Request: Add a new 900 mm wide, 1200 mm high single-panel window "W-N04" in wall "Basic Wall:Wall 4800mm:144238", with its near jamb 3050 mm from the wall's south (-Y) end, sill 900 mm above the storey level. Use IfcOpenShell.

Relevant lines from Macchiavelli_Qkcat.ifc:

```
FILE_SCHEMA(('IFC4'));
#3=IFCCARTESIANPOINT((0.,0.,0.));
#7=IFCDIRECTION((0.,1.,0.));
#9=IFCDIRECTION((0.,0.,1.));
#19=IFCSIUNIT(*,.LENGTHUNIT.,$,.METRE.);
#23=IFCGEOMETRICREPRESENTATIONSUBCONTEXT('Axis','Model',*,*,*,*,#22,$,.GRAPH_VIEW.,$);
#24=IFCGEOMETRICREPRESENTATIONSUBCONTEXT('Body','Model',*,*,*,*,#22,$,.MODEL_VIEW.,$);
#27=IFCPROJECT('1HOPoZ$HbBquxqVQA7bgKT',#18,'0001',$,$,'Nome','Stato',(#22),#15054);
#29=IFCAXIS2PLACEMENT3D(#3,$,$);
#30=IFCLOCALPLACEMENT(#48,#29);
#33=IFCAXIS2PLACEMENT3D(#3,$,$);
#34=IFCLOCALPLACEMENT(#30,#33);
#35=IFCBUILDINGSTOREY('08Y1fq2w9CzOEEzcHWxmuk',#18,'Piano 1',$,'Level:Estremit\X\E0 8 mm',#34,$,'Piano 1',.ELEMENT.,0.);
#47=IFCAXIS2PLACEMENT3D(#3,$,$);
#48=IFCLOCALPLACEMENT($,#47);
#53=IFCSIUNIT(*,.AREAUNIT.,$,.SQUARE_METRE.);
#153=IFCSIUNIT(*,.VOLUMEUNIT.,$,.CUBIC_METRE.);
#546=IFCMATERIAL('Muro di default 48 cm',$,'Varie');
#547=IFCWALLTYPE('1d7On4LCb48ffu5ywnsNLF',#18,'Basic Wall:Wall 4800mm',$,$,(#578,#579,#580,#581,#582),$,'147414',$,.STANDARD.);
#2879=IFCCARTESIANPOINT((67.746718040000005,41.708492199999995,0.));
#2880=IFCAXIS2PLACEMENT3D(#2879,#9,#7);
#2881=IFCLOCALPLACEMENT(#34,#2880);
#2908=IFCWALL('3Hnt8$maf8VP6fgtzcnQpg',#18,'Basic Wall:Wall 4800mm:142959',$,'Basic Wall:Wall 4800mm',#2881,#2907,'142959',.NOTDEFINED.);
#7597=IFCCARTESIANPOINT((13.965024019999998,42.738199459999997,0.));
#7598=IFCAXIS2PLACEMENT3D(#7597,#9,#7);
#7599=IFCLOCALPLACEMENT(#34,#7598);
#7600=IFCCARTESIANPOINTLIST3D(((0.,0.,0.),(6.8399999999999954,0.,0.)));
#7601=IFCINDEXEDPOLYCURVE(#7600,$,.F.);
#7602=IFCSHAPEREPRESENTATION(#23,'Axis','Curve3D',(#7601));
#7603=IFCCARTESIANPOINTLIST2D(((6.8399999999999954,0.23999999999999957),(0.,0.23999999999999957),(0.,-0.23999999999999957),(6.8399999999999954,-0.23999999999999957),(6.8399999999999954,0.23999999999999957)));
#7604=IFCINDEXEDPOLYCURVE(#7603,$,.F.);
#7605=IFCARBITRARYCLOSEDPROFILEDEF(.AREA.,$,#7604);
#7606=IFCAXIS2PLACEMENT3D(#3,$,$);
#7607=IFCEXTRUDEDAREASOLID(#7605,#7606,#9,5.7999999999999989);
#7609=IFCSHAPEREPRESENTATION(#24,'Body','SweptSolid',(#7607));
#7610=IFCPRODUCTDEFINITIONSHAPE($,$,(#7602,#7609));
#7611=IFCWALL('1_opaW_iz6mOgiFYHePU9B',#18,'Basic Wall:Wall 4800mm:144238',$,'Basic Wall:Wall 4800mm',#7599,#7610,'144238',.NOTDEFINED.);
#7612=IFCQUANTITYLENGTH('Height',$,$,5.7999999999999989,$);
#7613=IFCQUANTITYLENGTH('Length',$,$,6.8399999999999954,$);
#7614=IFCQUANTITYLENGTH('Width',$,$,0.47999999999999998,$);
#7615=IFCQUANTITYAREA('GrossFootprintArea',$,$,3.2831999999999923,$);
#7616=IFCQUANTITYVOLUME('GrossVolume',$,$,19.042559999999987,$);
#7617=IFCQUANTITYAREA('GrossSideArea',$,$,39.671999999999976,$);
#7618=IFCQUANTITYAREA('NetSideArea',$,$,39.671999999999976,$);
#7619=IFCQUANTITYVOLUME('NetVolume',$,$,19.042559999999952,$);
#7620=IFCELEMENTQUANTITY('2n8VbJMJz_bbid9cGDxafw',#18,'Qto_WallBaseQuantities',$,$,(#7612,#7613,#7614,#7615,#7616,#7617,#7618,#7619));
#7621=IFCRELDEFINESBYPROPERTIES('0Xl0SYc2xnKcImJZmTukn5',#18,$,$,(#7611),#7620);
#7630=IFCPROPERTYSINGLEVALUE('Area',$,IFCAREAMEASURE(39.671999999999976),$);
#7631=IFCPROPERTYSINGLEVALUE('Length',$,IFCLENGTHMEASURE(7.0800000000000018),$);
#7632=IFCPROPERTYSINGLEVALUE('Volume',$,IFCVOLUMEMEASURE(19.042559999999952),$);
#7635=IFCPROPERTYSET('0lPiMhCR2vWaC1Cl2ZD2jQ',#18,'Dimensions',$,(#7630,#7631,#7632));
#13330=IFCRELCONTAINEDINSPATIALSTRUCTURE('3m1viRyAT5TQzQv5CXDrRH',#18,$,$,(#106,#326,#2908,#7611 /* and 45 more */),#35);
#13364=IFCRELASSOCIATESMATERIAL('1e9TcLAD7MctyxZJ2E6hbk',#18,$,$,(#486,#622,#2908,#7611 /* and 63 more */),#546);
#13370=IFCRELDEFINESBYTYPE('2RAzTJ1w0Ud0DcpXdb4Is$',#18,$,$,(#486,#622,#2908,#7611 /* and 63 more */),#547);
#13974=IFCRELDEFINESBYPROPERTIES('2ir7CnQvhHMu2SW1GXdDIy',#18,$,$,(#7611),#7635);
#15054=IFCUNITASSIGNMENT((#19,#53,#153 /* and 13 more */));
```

```python
import numpy as np
import ifcopenshell
import ifcopenshell.api.feature
import ifcopenshell.api.geometry
import ifcopenshell.api.pset
import ifcopenshell.api.root
import ifcopenshell.api.spatial
import ifcopenshell.geom
import ifcopenshell.util.element
import ifcopenshell.util.placement
import ifcopenshell.util.representation
import ifcopenshell.util.shape
import ifcopenshell.util.unit

model = ifcopenshell.open("Macchiavelli_Qkcat.ifc")
unit_scale = ifcopenshell.util.unit.calculate_unit_scale(model)
area_scale = ifcopenshell.util.unit.calculate_unit_scale(model, "AREAUNIT")
volume_scale = ifcopenshell.util.unit.calculate_unit_scale(model, "VOLUMEUNIT")
settings = ifcopenshell.geom.settings()


def volume(element):
    """Net volume in cubic metres, openings subtracted."""
    shape = ifcopenshell.geom.create_shape(settings, element)
    return ifcopenshell.util.shape.get_volume(shape.geometry)


wall = model.by_guid("1_opaW_iz6mOgiFYHePU9B")
storey = ifcopenshell.util.element.get_container(wall, ifc_class="IfcBuildingStorey")
context = ifcopenshell.util.representation.get_context(model, "Model", "Body", "MODEL_VIEW")
before = volume(wall)

width, height, from_end, sill = 0.9, 1.2, 3.05, 0.9  # metres

# The wall runs along its own X axis, and the end named is its -X end.
wall_shape = ifcopenshell.geom.create_shape(settings, wall)
x, y, z = ifcopenshell.util.shape.get_vertices(wall_shape.geometry).T
start = x.min() + from_end
face, thickness = float(y.min()), float(y.max() - y.min())
wall_matrix = ifcopenshell.util.placement.get_local_placement(wall.ObjectPlacement)
level = ifcopenshell.util.placement.get_local_placement(storey.ObjectPlacement)[2, 3]


def in_wall(x, y):
    """Placement at x, y metres in the wall's axes, at sill height."""
    matrix = wall_matrix.copy()
    matrix[:, 3] = wall_matrix @ np.array([x / unit_scale, y / unit_scale, 0.0, 1.0])
    matrix[2, 3] = level + sill / unit_scale
    return matrix


# Opening: a box that overshoots both wall faces by 50 mm.
opening = ifcopenshell.api.root.create_entity(model, ifc_class="IfcOpeningElement", predefined_type="OPENING")
box = ifcopenshell.api.geometry.add_wall_representation(
    model, context=context, length=width, height=height, thickness=thickness + 0.1
)
ifcopenshell.api.geometry.assign_representation(model, product=opening, representation=box)
ifcopenshell.api.geometry.edit_object_placement(model, product=opening, matrix=in_wall(start, face - 0.05), is_si=False)
ifcopenshell.api.feature.add_feature(model, feature=opening, element=wall)

window = ifcopenshell.api.root.create_entity(model, ifc_class="IfcWindow", name="W-N04", predefined_type="WINDOW")
window.OverallWidth, window.OverallHeight = width / unit_scale, height / unit_scale
window.PartitioningType = "SINGLE_PANEL"
body = ifcopenshell.api.geometry.add_window_representation(
    model,
    context=context,
    overall_width=window.OverallWidth,
    overall_height=window.OverallHeight,
    partition_type="SINGLE_PANEL",
)
ifcopenshell.api.geometry.assign_representation(model, product=window, representation=body)
ifcopenshell.api.spatial.assign_container(model, products=[window], relating_structure=storey)
ifcopenshell.api.feature.add_filling(model, opening=opening, element=window)

# Centre the window in the wall's thickness.
ifcopenshell.api.geometry.edit_object_placement(model, product=window, matrix=in_wall(start, face), is_si=False)
window_shape = ifcopenshell.geom.create_shape(settings, window)
depth = ifcopenshell.util.shape.get_vertices(window_shape.geometry)[:, 1]
offset = face + thickness / 2 - (depth.min() + depth.max()) / 2
ifcopenshell.api.geometry.edit_object_placement(model, product=window, matrix=in_wall(start, offset), is_si=False)

after = volume(wall)

# Update the wall's stored quantities.
qto = model.by_id(ifcopenshell.util.element.get_pset(wall, "Qto_WallBaseQuantities", should_inherit=False)["id"])
ifcopenshell.api.pset.edit_qto(model, qto=qto, properties={
    "NetSideArea": after / thickness / area_scale,
    "NetVolume": after / volume_scale,
})
pset = model.by_id(ifcopenshell.util.element.get_pset(wall, "Dimensions", should_inherit=False)["id"])
ifcopenshell.api.pset.edit_pset(model, pset=pset, properties={
    "Area": model.create_entity("IfcAreaMeasure", after / thickness / area_scale),
    "Volume": model.create_entity("IfcVolumeMeasure", after / volume_scale),
})

print(f"wall volume {before:.3f} -> {after:.3f} m3")

model.write("Macchiavelli_Qkcat_rev.ifc")
```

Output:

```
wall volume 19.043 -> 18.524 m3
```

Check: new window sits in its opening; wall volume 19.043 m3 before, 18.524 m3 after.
